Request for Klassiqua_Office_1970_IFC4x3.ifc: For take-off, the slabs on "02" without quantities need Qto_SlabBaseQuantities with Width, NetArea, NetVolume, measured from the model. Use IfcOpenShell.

First a look at what the model holds.

```python
import ifcopenshell
import ifcopenshell.util.element
import ifcopenshell.util.unit

model = ifcopenshell.open("Klassiqua_Office_1970_IFC4x3.ifc")
print(model.schema)
for unit_type in ("LENGTHUNIT", "AREAUNIT", "VOLUMEUNIT"):
    print(unit_type, ifcopenshell.util.unit.calculate_unit_scale(model, unit_type))
storey = next(s for s in model.by_type("IfcBuildingStorey") if s.Name == "02")
slabs = [e for e in ifcopenshell.util.element.get_decomposition(storey) if e.is_a("IfcSlab")]
for e in sorted(slabs, key=lambda e: e.id()):
    print(e.id(), e.is_a(), e.Name, list(ifcopenshell.util.element.get_psets(e, qtos_only=True)), sep=" | ")
```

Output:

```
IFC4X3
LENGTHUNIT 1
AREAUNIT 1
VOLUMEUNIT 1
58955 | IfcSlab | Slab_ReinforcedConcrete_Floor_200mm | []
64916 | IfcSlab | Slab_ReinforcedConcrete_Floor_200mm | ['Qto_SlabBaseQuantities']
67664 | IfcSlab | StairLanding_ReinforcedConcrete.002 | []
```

```python
import ifcopenshell
import ifcopenshell.api.pset
import ifcopenshell.geom
import ifcopenshell.util.element
import ifcopenshell.util.shape
import ifcopenshell.util.unit

model = ifcopenshell.open("Klassiqua_Office_1970_IFC4x3.ifc")
unit_scale = ifcopenshell.util.unit.calculate_unit_scale(model)
area_scale = ifcopenshell.util.unit.calculate_unit_scale(model, "AREAUNIT")
volume_scale = ifcopenshell.util.unit.calculate_unit_scale(model, "VOLUMEUNIT")
settings = ifcopenshell.geom.settings()

storey = next(s for s in model.by_type("IfcBuildingStorey") if s.Name == "02")
slabs = [e for e in ifcopenshell.util.element.get_decomposition(storey) if e.is_a("IfcSlab")]

for e in sorted(slabs, key=lambda e: e.id()):
    if ifcopenshell.util.element.get_psets(e, qtos_only=True, should_inherit=False):
        continue
    # Geometry comes back in metres, in the element's own axes.
    shape = ifcopenshell.geom.create_shape(settings, e)
    values = {
        "Width": ifcopenshell.util.shape.get_z(shape.geometry) / unit_scale,
        "NetArea": ifcopenshell.util.shape.get_footprint_area(shape.geometry) / area_scale,
        "NetVolume": ifcopenshell.util.shape.get_volume(shape.geometry) / volume_scale,
    }
    qto = ifcopenshell.api.pset.add_qto(model, product=e, name="Qto_SlabBaseQuantities")
    ifcopenshell.api.pset.edit_qto(model, qto=qto, properties=values)
    print(e.id(), {k: round(v, 3) for k, v in values.items()})

model.write("Klassiqua_Office_1970_IFC4x3-out.ifc")
```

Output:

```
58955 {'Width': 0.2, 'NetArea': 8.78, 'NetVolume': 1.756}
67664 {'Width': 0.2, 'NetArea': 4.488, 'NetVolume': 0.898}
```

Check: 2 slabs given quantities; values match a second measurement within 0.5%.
